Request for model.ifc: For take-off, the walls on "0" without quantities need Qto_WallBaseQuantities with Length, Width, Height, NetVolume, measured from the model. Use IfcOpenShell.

First a look at what the model holds.

```python
import ifcopenshell
import ifcopenshell.util.element
import ifcopenshell.util.unit

model = ifcopenshell.open("model.ifc")
print(model.schema)
for unit_type in ("LENGTHUNIT", "AREAUNIT", "VOLUMEUNIT"):
    print(unit_type, ifcopenshell.util.unit.calculate_unit_scale(model, unit_type))
storey = next(s for s in model.by_type("IfcBuildingStorey") if s.Name == "0")
walls = [e for e in ifcopenshell.util.element.get_decomposition(storey) if e.is_a("IfcWall")]
for e in sorted(walls, key=lambda e: e.id()):
    print(e.id(), e.is_a(), e.Name, list(ifcopenshell.util.element.get_psets(e, qtos_only=True)), sep=" | ")
```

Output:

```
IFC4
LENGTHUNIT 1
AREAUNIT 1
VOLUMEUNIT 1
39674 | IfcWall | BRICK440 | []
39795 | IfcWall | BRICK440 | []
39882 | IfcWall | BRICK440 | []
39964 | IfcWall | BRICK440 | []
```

```python
import ifcopenshell
import ifcopenshell.api.pset
import ifcopenshell.geom
import ifcopenshell.util.element
import ifcopenshell.util.shape
import ifcopenshell.util.unit

model = ifcopenshell.open("model.ifc")
unit_scale = ifcopenshell.util.unit.calculate_unit_scale(model)
volume_scale = ifcopenshell.util.unit.calculate_unit_scale(model, "VOLUMEUNIT")
settings = ifcopenshell.geom.settings()

storey = next(s for s in model.by_type("IfcBuildingStorey") if s.Name == "0")
walls = [e for e in ifcopenshell.util.element.get_decomposition(storey) if e.is_a("IfcWall")]

for e in sorted(walls, key=lambda e: e.id()):
    if ifcopenshell.util.element.get_psets(e, qtos_only=True, should_inherit=False):
        continue
    # Geometry comes back in metres, in the element's own axes.
    shape = ifcopenshell.geom.create_shape(settings, e)
    values = {
        "Length": ifcopenshell.util.shape.get_x(shape.geometry) / unit_scale,
        "Width": ifcopenshell.util.shape.get_y(shape.geometry) / unit_scale,
        "Height": ifcopenshell.util.shape.get_z(shape.geometry) / unit_scale,
        "NetVolume": ifcopenshell.util.shape.get_volume(shape.geometry) / volume_scale,
    }
    qto = ifcopenshell.api.pset.add_qto(model, product=e, name="Qto_WallBaseQuantities")
    ifcopenshell.api.pset.edit_qto(model, qto=qto, properties=values)
    print(e.id(), {k: round(v, 3) for k, v in values.items()})

model.write("model_rev.ifc")
```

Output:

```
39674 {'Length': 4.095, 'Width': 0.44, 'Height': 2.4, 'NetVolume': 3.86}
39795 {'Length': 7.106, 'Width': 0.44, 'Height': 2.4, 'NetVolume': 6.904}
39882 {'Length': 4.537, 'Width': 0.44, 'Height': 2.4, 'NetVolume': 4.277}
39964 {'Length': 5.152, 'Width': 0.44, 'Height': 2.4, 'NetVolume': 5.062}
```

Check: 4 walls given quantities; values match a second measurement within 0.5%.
